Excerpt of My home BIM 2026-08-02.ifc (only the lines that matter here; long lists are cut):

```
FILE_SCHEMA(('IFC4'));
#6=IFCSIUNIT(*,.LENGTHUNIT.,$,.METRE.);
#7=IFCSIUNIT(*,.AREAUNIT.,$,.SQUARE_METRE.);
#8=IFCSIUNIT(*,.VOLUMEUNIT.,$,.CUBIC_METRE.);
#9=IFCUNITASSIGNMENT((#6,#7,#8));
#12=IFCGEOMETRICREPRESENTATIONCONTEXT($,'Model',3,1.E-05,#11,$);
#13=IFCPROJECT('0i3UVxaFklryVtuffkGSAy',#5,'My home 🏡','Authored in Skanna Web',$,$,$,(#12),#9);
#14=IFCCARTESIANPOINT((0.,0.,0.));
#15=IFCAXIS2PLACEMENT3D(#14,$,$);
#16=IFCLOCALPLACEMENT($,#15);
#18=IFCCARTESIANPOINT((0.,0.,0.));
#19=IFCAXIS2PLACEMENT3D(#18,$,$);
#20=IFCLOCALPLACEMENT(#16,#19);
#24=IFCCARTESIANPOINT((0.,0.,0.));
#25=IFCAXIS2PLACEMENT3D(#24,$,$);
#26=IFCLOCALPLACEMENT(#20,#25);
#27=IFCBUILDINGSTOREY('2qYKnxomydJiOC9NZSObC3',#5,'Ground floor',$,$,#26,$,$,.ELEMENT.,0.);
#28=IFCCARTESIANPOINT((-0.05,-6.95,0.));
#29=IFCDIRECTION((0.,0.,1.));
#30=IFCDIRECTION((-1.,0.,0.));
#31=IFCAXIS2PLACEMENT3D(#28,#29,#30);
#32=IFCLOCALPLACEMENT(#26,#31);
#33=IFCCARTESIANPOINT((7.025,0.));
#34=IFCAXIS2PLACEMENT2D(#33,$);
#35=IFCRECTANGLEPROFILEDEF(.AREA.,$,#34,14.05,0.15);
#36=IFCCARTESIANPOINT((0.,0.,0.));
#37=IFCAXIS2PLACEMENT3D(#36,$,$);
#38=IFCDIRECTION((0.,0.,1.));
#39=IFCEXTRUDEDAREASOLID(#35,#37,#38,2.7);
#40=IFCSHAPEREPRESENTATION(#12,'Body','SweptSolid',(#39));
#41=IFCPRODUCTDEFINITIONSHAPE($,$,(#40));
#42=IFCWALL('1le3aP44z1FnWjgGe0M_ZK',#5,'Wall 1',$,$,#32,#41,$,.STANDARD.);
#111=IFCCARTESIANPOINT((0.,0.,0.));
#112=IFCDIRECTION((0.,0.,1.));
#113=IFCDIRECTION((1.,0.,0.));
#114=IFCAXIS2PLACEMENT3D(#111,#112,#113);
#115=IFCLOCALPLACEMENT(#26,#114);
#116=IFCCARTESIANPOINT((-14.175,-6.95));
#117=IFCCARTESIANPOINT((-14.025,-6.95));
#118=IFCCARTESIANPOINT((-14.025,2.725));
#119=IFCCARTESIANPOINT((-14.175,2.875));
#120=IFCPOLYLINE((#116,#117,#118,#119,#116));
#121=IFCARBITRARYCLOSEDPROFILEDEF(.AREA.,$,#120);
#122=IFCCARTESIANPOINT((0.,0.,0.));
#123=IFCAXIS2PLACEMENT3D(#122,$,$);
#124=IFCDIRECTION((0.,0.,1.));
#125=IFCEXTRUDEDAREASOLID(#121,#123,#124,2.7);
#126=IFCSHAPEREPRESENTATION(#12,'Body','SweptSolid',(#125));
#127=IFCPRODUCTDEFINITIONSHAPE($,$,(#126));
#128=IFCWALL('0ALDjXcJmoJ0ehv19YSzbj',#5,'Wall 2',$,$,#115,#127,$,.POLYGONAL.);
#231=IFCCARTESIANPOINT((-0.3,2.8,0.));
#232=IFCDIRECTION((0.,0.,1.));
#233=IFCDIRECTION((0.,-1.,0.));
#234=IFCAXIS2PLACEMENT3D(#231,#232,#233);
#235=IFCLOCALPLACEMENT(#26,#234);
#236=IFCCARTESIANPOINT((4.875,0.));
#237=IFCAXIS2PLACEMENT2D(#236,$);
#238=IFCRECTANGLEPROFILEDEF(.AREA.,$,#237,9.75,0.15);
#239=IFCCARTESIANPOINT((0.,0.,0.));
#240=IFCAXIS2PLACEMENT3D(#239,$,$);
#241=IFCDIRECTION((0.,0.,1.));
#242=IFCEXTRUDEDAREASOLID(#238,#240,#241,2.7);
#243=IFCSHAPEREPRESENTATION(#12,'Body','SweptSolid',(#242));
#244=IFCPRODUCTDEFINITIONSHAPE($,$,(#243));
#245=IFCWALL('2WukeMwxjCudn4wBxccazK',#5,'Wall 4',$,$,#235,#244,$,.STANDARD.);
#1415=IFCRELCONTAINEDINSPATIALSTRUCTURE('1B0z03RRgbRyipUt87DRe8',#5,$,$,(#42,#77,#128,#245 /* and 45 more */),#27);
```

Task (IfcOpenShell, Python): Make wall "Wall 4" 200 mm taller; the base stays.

```python
import ifcopenshell
import ifcopenshell.geom
import ifcopenshell.util.shape

model = ifcopenshell.open("My home BIM 2026-08-02.ifc")
settings = ifcopenshell.geom.settings()


def volume(element):
    """Net volume in cubic metres, openings subtracted."""
    shape = ifcopenshell.geom.create_shape(settings, element)
    return ifcopenshell.util.shape.get_volume(shape.geometry)


wall = model.by_id(245)
before = volume(wall)

body = next(r for r in wall.Representation.Representations if r.RepresentationIdentifier == "Body")
solid = body.Items[0]
old_height = solid.Depth
solid.Depth += 0.2
after = volume(wall)

print(f"height {old_height:g} -> {solid.Depth:g}, volume {before:.3f} -> {after:.3f} m3")

model.write("My home BIM 2026-08-02_edited.ifc")
```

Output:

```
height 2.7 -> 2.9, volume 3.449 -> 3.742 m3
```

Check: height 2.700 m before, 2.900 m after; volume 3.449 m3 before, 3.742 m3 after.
